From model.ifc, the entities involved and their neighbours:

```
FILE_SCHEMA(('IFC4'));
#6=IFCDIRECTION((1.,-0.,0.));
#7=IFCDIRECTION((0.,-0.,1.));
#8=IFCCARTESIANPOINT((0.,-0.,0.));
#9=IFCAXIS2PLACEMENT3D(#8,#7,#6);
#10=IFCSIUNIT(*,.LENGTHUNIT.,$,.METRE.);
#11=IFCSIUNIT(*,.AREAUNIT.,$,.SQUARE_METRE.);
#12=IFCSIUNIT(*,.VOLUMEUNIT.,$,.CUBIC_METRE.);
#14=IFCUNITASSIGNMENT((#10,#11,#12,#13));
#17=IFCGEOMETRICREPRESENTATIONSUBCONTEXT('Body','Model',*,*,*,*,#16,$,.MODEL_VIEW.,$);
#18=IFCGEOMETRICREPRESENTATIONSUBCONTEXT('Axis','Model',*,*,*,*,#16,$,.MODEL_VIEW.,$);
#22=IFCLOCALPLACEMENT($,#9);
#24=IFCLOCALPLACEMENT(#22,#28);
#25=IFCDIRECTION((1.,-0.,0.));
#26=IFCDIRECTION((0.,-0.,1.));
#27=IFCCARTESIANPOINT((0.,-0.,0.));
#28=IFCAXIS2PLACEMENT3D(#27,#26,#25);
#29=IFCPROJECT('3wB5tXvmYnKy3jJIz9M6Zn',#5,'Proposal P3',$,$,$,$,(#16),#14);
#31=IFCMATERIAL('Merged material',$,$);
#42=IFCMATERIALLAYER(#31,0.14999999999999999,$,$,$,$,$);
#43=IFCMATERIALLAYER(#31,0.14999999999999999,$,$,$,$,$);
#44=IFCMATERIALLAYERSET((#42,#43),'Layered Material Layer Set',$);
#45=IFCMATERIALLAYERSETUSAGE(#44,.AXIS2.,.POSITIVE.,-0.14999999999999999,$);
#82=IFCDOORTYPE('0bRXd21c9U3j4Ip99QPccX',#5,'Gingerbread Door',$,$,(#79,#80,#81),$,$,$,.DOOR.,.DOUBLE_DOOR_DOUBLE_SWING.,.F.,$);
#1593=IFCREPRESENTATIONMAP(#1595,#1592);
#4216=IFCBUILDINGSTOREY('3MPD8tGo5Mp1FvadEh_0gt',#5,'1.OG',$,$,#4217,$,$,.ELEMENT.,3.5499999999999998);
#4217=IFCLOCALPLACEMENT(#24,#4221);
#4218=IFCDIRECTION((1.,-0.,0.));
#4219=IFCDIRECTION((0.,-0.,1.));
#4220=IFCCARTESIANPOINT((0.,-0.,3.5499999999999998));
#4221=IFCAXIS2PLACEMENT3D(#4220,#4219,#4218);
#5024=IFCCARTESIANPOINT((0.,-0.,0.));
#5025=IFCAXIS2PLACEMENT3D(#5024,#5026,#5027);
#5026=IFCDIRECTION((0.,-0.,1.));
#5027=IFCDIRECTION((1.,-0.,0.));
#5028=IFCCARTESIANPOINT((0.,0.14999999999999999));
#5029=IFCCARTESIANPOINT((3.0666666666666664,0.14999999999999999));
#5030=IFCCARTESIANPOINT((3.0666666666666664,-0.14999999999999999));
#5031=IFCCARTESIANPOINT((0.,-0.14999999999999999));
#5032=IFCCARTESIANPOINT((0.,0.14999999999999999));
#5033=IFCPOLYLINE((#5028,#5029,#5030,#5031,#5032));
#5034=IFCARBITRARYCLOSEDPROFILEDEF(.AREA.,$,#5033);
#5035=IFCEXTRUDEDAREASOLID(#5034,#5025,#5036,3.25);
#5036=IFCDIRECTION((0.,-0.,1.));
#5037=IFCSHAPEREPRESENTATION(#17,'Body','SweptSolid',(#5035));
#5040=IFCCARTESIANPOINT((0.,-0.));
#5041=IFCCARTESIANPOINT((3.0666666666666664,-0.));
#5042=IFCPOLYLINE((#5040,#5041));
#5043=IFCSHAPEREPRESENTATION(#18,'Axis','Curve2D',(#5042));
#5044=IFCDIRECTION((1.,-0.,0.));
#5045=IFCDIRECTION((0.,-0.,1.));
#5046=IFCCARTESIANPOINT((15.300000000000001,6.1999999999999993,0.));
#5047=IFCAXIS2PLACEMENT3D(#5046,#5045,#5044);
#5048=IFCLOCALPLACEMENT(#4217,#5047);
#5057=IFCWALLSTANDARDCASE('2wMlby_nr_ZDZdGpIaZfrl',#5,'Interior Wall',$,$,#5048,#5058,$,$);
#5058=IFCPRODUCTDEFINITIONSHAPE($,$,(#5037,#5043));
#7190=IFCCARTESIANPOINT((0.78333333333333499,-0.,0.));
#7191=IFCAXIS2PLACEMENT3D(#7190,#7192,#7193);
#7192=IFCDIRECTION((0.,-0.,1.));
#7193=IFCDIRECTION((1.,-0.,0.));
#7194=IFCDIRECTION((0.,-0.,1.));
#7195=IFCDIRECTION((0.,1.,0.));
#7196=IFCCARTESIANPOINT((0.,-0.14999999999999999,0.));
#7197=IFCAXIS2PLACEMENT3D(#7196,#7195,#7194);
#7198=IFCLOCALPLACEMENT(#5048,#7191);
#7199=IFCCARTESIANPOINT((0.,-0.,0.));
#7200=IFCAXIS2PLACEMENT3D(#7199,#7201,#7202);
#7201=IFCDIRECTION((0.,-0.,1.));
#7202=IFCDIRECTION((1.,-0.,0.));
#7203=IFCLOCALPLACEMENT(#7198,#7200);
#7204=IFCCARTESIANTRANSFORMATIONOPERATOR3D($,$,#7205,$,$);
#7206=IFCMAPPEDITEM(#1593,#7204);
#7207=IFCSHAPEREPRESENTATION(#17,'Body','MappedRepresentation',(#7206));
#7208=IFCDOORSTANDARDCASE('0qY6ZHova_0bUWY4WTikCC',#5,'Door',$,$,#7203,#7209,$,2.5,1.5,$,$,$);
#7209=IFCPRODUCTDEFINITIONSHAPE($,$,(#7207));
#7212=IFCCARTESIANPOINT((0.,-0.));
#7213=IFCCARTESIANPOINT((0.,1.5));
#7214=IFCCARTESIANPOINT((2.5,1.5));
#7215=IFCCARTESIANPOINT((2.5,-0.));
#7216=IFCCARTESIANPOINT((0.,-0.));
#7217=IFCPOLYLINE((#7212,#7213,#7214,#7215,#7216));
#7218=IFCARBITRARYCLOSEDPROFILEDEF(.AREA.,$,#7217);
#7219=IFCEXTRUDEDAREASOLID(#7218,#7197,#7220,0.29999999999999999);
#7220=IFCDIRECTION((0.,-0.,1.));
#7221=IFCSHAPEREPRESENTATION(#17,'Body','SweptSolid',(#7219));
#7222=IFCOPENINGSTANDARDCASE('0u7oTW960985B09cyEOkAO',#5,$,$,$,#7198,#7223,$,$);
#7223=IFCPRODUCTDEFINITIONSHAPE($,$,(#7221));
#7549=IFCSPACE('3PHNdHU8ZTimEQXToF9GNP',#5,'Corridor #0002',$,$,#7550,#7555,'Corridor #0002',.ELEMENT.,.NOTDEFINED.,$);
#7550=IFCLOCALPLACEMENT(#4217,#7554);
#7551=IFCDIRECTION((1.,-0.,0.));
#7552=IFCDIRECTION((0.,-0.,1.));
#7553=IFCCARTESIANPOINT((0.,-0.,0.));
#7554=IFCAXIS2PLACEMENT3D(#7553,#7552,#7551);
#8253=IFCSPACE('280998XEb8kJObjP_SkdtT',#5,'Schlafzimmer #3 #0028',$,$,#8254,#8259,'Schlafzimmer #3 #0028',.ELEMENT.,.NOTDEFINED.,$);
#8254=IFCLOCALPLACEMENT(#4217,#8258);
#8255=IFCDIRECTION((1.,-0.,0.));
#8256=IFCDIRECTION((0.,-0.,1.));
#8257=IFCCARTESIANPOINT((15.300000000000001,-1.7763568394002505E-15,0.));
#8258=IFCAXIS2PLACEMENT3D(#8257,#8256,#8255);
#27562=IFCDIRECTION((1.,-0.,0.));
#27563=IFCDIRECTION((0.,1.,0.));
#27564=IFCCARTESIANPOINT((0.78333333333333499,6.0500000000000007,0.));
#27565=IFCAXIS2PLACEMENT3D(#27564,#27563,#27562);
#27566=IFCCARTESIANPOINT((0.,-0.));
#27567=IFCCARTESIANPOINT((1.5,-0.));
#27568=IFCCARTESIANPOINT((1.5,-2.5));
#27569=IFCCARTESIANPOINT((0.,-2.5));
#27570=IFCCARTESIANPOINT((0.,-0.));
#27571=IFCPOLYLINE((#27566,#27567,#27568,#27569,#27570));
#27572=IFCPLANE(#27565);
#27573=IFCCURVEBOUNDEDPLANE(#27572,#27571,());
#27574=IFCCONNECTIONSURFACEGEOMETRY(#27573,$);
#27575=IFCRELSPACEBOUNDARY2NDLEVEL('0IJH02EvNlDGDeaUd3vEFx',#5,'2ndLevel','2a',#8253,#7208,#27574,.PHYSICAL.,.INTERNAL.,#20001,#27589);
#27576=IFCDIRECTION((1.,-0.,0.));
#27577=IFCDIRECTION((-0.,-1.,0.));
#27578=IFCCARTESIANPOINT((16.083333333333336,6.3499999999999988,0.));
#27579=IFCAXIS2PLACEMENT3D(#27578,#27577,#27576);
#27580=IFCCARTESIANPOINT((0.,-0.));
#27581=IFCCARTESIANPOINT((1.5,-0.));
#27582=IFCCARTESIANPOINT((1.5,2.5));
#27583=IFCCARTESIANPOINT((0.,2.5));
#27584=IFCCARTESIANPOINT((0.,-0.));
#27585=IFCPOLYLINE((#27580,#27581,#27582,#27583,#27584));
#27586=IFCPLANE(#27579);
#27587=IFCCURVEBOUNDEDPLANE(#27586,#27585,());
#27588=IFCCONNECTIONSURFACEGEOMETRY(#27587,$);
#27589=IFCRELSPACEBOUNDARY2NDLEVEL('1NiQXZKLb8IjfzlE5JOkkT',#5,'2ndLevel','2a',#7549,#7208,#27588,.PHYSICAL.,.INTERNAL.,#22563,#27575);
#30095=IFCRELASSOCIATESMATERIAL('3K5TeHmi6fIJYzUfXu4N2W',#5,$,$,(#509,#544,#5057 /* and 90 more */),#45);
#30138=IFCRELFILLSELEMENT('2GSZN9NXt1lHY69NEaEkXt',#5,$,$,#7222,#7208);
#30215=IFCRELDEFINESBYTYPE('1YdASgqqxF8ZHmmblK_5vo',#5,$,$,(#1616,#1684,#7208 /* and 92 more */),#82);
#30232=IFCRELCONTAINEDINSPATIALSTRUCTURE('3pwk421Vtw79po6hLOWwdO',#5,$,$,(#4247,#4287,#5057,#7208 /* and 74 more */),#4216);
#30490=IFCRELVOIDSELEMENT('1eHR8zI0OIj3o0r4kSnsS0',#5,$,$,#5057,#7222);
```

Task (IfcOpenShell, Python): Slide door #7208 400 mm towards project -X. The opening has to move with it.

```python
import numpy as np
import ifcopenshell
import ifcopenshell.api.geometry
import ifcopenshell.util.placement
import ifcopenshell.util.unit

model = ifcopenshell.open("model.ifc")
unit_scale = ifcopenshell.util.unit.calculate_unit_scale(model)

door = model.by_guid("0qY6ZHova_0bUWY4WTikCC")
opening = door.FillsVoids[0].RelatingOpeningElement
wall = opening.VoidsElements[0].RelatingBuildingElement

wall_matrix = ifcopenshell.util.placement.get_local_placement(wall.ObjectPlacement)
shift = wall_matrix[:3, 0] * -0.4 / unit_scale
before = ifcopenshell.util.placement.get_local_placement(door.ObjectPlacement)[:3, 3].copy()

# The door is placed relative to its opening, so it follows when the opening moves.
matrix = ifcopenshell.util.placement.get_local_placement(opening.ObjectPlacement)
matrix[:3, 3] += shift
ifcopenshell.api.geometry.edit_object_placement(
    model, product=opening, matrix=matrix, is_si=False, should_transform_children=True
)

# Space boundary surfaces are stored in each space's coordinates; move them too.
for rel in door.ProvidesBoundaries:
    if not rel.ConnectionGeometry:
        continue
    surface = rel.ConnectionGeometry.SurfaceOnRelatingElement.BasisSurface
    space_matrix = ifcopenshell.util.placement.get_local_placement(rel.RelatingSpace.ObjectPlacement)
    point = np.array(surface.Position.Location.Coordinates) + space_matrix[:3, :3].T @ shift
    surface.Position = model.createIfcAxis2Placement3D(
        model.createIfcCartesianPoint(point.tolist()), surface.Position.Axis, surface.Position.RefDirection
    )

after = ifcopenshell.util.placement.get_local_placement(door.ObjectPlacement)[:3, 3]
print("door moved by", (after - before).round(3) + 0.0)

model.write("model_rev.ifc")
```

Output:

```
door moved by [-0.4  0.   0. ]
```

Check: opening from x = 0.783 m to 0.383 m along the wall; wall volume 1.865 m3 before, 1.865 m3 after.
